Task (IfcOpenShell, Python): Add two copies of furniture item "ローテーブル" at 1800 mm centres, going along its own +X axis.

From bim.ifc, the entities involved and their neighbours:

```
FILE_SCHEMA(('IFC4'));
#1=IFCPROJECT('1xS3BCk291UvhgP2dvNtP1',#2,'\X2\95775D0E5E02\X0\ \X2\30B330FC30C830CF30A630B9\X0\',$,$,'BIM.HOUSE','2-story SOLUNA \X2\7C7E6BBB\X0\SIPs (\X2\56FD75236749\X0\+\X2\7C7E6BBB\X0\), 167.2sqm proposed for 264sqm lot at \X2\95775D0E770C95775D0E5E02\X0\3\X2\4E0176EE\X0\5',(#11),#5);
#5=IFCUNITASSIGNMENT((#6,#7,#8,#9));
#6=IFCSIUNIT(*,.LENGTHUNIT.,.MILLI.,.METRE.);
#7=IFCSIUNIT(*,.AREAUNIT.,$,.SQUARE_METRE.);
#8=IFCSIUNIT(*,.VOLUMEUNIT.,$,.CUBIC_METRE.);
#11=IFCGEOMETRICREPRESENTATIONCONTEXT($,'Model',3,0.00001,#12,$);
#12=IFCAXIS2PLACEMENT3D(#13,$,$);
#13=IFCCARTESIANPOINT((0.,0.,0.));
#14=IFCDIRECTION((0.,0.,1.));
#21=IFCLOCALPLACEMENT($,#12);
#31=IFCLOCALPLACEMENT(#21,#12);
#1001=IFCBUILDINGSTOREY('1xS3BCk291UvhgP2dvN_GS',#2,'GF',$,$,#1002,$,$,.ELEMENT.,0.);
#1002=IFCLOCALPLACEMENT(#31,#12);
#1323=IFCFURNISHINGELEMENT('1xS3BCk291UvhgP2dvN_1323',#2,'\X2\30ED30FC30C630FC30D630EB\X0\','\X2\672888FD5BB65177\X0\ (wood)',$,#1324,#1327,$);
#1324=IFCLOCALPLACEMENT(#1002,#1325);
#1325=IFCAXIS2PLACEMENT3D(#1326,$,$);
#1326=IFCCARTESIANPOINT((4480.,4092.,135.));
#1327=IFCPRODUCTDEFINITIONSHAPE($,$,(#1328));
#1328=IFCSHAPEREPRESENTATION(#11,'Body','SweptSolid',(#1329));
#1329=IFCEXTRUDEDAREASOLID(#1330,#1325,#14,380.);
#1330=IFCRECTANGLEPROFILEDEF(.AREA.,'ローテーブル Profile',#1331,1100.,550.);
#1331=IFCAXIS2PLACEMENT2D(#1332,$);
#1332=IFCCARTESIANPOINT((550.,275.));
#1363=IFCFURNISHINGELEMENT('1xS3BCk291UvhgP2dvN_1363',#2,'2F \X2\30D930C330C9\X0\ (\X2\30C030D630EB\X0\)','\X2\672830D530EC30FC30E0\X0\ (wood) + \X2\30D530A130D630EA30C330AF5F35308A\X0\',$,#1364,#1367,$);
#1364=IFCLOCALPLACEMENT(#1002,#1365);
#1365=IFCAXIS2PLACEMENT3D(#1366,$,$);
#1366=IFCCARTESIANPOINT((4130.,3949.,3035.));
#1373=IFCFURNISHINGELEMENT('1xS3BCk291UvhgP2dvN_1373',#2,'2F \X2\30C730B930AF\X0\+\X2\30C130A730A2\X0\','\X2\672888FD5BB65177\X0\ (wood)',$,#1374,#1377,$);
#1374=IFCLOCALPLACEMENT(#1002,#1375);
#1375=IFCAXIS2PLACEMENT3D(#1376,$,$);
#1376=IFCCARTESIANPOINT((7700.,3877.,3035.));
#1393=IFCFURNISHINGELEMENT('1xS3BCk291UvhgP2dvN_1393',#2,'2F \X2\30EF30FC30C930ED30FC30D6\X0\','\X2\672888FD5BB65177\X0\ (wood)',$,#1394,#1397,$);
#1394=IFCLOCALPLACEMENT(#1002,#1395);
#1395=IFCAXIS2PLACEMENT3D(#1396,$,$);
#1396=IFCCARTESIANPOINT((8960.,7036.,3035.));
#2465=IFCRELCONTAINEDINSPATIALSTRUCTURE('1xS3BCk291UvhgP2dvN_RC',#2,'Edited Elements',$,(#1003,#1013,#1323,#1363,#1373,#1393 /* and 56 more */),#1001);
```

```python
import ifcopenshell
import ifcopenshell.api.geometry
import ifcopenshell.api.root
import ifcopenshell.util.element
import ifcopenshell.util.placement
import ifcopenshell.util.unit

model = ifcopenshell.open("bim.ifc")
unit_scale = ifcopenshell.util.unit.calculate_unit_scale(model)


def reuse_history(source, copy):
    """copy_class also copies each property set's owner history, people and application; keep the originals."""
    for rel in copy.IsDefinedBy:
        if rel.is_a("IfcRelDefinesByProperties") and (history := rel.RelatingPropertyDefinition.OwnerHistory):
            rel.RelatingPropertyDefinition.OwnerHistory = source.OwnerHistory
            ifcopenshell.util.element.remove_deep2(model, history)


source = model.by_guid("1xS3BCk291UvhgP2dvN_1323")
base = ifcopenshell.util.placement.get_local_placement(source.ObjectPlacement)
step = base[:3, 0] * 1.8 / unit_scale

for i in range(1, 3):
    copy = ifcopenshell.api.root.copy_class(model, product=source)
    copy.Representation = ifcopenshell.util.element.copy_deep(
        model, source.Representation, exclude=["IfcGeometricRepresentationContext", "IfcRepresentationMap"]
    )
    reuse_history(source, copy)
    matrix = base.copy()
    matrix[:3, 3] += i * step
    print("added at", matrix[:3, 3].round(3) + 0.0)
    ifcopenshell.api.geometry.edit_object_placement(model, product=copy, matrix=matrix, is_si=False)

model.write("bim_rev.ifc")
```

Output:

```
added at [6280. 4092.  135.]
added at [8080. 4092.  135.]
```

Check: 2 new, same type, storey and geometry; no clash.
